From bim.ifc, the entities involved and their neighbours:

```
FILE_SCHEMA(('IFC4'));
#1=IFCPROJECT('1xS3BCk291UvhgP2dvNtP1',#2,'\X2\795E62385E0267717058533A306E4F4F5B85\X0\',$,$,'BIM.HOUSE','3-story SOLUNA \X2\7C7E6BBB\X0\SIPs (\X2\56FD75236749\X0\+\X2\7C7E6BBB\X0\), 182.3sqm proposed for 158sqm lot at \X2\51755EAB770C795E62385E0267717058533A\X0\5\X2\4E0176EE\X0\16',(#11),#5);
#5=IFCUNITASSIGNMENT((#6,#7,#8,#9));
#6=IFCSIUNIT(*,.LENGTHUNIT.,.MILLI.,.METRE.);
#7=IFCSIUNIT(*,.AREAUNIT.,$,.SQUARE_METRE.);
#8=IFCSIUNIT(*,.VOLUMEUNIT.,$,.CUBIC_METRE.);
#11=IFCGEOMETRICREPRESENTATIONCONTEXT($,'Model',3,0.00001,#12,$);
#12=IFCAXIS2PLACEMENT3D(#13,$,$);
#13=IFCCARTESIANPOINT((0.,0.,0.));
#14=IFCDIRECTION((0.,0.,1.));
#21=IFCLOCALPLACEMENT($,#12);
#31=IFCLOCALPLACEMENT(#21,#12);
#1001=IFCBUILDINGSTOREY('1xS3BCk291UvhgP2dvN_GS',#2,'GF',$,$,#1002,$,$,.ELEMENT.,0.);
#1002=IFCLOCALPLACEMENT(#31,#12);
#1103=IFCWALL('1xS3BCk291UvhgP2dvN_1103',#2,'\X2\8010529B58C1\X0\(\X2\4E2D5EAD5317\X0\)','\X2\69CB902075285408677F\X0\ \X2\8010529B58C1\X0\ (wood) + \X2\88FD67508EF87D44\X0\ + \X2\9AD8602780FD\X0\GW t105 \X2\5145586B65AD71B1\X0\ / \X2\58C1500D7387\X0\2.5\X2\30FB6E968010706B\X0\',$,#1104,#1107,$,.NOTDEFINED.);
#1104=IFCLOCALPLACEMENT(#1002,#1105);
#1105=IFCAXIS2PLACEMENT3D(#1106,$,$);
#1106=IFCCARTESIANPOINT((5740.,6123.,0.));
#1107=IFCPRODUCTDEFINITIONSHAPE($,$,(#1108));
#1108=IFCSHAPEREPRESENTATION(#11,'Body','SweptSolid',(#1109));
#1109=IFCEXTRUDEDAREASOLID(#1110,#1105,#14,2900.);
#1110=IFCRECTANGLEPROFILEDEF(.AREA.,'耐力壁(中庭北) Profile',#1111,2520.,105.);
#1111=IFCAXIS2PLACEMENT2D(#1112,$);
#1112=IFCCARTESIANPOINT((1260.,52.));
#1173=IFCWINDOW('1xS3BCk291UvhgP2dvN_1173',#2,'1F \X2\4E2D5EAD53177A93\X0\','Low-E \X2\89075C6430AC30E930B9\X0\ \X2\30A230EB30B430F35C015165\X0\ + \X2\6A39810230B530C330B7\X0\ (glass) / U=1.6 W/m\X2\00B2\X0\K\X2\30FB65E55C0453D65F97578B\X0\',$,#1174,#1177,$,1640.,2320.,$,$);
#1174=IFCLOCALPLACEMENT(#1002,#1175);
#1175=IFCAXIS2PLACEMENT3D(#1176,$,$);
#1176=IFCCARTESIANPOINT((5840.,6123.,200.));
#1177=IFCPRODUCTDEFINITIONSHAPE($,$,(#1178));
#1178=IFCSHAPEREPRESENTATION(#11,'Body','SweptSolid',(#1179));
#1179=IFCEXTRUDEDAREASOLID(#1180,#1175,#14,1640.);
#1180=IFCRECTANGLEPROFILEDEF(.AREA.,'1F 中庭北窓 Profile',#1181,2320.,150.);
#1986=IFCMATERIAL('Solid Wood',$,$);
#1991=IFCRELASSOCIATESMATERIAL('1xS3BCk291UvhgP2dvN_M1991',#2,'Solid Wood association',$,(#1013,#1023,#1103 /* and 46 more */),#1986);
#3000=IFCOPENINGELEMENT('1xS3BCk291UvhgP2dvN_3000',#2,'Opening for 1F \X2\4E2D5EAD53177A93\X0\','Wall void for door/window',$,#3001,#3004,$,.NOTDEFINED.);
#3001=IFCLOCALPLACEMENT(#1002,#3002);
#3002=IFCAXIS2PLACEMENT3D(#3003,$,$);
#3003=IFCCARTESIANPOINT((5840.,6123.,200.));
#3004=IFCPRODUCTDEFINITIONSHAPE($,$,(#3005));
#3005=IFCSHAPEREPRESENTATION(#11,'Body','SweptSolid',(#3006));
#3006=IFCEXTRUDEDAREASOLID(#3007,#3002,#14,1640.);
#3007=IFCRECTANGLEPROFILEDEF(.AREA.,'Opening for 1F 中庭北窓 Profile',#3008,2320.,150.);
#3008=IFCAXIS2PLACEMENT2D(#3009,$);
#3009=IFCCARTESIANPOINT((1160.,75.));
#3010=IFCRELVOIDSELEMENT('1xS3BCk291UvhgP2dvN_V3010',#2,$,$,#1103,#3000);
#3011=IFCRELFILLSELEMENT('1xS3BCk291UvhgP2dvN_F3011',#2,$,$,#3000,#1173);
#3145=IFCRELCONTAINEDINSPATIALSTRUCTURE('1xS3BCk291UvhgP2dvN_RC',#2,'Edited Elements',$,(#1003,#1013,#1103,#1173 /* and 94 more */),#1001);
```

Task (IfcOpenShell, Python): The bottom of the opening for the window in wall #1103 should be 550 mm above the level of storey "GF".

```python
import numpy as np
import ifcopenshell
import ifcopenshell.api.geometry
import ifcopenshell.geom
import ifcopenshell.util.element
import ifcopenshell.util.placement
import ifcopenshell.util.shape
import ifcopenshell.util.unit

model = ifcopenshell.open("bim.ifc")
unit_scale = ifcopenshell.util.unit.calculate_unit_scale(model)

window = model.by_guid("1xS3BCk291UvhgP2dvN_1173")
opening = window.FillsVoids[0].RelatingOpeningElement
storey = ifcopenshell.util.element.get_container(window, ifc_class="IfcBuildingStorey")
level = ifcopenshell.util.placement.get_local_placement(storey.ObjectPlacement)[2, 3]

# The opening's origin need not be at the sill, so measure its lowest point.
shape = ifcopenshell.geom.create_shape(ifcopenshell.geom.settings(), opening)
bottom = ifcopenshell.util.shape.get_shape_bottom_elevation(shape, shape.geometry) / unit_scale
dz = level + 550.0 - bottom

shift = np.array([0.0, 0.0, dz])
# The window is not placed relative to its opening, so move both.
for product in (opening, window):
    matrix = ifcopenshell.util.placement.get_local_placement(product.ObjectPlacement)
    matrix[:3, 3] += shift
    ifcopenshell.api.geometry.edit_object_placement(model, product=product, matrix=matrix, is_si=False)

print(f"moved by {dz * unit_scale:+.3f} m")

model.write("bim_v2.ifc")
```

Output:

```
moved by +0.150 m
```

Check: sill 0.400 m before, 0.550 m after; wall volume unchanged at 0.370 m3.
